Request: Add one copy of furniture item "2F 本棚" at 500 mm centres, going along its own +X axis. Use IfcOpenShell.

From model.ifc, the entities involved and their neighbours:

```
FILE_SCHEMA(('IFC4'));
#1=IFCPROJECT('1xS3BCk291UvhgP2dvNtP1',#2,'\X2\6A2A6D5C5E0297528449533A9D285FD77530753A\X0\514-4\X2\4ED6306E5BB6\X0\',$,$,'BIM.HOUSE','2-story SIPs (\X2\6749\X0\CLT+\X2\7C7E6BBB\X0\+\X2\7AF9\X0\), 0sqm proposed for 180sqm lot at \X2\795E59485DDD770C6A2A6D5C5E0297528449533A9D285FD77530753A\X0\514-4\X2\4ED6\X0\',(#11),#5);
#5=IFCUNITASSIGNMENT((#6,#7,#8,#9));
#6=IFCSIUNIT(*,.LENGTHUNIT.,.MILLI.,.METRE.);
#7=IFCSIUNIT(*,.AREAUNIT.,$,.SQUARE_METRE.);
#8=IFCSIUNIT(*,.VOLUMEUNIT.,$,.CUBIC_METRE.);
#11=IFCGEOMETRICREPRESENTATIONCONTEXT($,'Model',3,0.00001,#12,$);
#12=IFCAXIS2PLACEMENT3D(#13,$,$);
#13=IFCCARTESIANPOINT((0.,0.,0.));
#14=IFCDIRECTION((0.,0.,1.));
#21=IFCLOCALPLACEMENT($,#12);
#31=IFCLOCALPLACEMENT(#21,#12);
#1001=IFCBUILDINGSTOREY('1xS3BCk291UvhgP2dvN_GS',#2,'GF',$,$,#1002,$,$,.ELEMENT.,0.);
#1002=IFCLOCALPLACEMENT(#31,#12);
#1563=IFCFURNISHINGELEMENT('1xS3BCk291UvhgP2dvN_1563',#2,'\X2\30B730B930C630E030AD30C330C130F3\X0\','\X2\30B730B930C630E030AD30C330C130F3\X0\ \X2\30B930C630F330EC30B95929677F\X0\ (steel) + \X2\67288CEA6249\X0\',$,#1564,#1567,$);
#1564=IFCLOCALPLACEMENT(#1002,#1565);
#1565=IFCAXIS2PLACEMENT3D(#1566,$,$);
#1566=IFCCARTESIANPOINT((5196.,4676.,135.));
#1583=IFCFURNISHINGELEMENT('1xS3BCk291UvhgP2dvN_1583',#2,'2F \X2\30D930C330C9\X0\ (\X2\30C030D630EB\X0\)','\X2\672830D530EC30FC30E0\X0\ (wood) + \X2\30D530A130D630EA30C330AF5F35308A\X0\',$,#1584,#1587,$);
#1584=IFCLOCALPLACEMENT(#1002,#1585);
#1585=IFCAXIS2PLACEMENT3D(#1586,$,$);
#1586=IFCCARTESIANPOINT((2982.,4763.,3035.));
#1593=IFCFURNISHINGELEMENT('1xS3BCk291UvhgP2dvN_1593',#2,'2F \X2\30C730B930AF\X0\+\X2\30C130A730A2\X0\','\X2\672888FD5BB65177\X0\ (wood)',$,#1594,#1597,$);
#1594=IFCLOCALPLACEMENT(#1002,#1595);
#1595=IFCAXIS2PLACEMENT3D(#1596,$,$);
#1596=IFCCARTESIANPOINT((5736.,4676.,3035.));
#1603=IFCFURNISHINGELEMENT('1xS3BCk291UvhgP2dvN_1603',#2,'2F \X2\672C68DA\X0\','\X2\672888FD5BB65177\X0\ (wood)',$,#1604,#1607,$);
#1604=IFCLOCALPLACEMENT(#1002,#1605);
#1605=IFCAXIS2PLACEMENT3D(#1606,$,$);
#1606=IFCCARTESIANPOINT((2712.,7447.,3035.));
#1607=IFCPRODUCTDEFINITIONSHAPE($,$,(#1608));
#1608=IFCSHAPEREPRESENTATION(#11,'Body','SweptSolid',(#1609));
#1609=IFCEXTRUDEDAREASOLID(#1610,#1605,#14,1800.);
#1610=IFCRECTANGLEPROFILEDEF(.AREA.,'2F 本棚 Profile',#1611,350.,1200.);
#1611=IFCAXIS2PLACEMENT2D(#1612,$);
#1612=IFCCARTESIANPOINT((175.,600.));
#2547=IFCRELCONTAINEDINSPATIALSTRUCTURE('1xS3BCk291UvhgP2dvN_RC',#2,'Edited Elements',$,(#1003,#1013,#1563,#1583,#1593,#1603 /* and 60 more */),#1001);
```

```python
import ifcopenshell
import ifcopenshell.api.geometry
import ifcopenshell.api.root
import ifcopenshell.util.element
import ifcopenshell.util.placement

model = ifcopenshell.open("model.ifc")


def reuse_history(source, copy):
    """copy_class also copies each property set's owner history, people and application; keep the originals."""
    for rel in copy.IsDefinedBy:
        if rel.is_a("IfcRelDefinesByProperties") and (history := rel.RelatingPropertyDefinition.OwnerHistory):
            rel.RelatingPropertyDefinition.OwnerHistory = source.OwnerHistory
            ifcopenshell.util.element.remove_deep2(model, history)


source = model.by_id(1603)
base = ifcopenshell.util.placement.get_local_placement(source.ObjectPlacement)
step = base[:3, 0] * 500.0

for i in range(1, 2):
    copy = ifcopenshell.api.root.copy_class(model, product=source)
    copy.Representation = ifcopenshell.util.element.copy_deep(
        model, source.Representation, exclude=["IfcGeometricRepresentationContext", "IfcRepresentationMap"]
    )
    reuse_history(source, copy)
    matrix = base.copy()
    matrix[:3, 3] += i * step
    print("added at", matrix[:3, 3].round(3) + 0.0)
    ifcopenshell.api.geometry.edit_object_placement(model, product=copy, matrix=matrix, is_si=False)

model.write("model-out.ifc")
```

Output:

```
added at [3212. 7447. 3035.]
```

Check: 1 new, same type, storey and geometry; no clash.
